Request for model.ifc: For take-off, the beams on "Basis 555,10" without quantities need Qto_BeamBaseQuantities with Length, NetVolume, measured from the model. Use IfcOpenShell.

First a look at what the model holds.

```python
import ifcopenshell
import ifcopenshell.util.element
import ifcopenshell.util.unit

model = ifcopenshell.open("model.ifc")
print(model.schema)
for unit_type in ("LENGTHUNIT", "AREAUNIT", "VOLUMEUNIT"):
    print(unit_type, ifcopenshell.util.unit.calculate_unit_scale(model, unit_type))
storey = next(s for s in model.by_type("IfcBuildingStorey") if s.Name == "Basis 555,10")
beams = [e for e in ifcopenshell.util.element.get_decomposition(storey) if e.is_a("IfcBeam")]
for e in sorted(beams, key=lambda e: e.id()):
    print(e.id(), e.is_a(), e.Name, list(ifcopenshell.util.element.get_psets(e, qtos_only=True)), sep=" | ")
```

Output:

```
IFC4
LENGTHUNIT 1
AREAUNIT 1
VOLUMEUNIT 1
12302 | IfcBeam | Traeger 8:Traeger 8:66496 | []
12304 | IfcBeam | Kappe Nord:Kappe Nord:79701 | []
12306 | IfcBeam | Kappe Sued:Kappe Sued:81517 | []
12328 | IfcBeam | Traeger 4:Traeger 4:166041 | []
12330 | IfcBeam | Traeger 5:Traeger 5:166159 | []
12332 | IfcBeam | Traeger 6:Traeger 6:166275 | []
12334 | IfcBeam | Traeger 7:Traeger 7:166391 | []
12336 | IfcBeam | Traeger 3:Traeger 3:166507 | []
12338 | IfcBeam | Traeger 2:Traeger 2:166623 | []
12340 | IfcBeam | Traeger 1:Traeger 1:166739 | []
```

```python
import ifcopenshell
import ifcopenshell.api.pset
import ifcopenshell.geom
import ifcopenshell.util.element
import ifcopenshell.util.shape
import ifcopenshell.util.unit

model = ifcopenshell.open("model.ifc")
unit_scale = ifcopenshell.util.unit.calculate_unit_scale(model)
volume_scale = ifcopenshell.util.unit.calculate_unit_scale(model, "VOLUMEUNIT")
settings = ifcopenshell.geom.settings()

storey = next(s for s in model.by_type("IfcBuildingStorey") if s.Name == "Basis 555,10")
beams = [e for e in ifcopenshell.util.element.get_decomposition(storey) if e.is_a("IfcBeam")]

for e in sorted(beams, key=lambda e: e.id()):
    if ifcopenshell.util.element.get_psets(e, qtos_only=True, should_inherit=False):
        continue
    # Geometry comes back in metres, in the element's own axes.
    shape = ifcopenshell.geom.create_shape(settings, e)
    values = {
        "Length": ifcopenshell.util.shape.get_max_xyz(shape.geometry) / unit_scale,
        "NetVolume": ifcopenshell.util.shape.get_volume(shape.geometry) / volume_scale,
    }
    qto = ifcopenshell.api.pset.add_qto(model, product=e, name="Qto_BeamBaseQuantities")
    ifcopenshell.api.pset.edit_qto(model, qto=qto, properties=values)
    print(e.id(), {k: round(v, 3) for k, v in values.items()})

model.write("model_v2.ifc")
```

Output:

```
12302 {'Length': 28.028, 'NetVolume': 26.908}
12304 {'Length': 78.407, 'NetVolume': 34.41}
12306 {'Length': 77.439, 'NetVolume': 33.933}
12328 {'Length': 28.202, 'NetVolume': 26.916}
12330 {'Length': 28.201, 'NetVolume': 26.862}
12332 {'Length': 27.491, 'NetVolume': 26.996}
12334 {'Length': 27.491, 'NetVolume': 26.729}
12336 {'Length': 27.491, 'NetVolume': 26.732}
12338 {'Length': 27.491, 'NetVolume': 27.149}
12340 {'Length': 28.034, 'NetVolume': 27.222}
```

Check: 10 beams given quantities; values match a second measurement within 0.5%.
